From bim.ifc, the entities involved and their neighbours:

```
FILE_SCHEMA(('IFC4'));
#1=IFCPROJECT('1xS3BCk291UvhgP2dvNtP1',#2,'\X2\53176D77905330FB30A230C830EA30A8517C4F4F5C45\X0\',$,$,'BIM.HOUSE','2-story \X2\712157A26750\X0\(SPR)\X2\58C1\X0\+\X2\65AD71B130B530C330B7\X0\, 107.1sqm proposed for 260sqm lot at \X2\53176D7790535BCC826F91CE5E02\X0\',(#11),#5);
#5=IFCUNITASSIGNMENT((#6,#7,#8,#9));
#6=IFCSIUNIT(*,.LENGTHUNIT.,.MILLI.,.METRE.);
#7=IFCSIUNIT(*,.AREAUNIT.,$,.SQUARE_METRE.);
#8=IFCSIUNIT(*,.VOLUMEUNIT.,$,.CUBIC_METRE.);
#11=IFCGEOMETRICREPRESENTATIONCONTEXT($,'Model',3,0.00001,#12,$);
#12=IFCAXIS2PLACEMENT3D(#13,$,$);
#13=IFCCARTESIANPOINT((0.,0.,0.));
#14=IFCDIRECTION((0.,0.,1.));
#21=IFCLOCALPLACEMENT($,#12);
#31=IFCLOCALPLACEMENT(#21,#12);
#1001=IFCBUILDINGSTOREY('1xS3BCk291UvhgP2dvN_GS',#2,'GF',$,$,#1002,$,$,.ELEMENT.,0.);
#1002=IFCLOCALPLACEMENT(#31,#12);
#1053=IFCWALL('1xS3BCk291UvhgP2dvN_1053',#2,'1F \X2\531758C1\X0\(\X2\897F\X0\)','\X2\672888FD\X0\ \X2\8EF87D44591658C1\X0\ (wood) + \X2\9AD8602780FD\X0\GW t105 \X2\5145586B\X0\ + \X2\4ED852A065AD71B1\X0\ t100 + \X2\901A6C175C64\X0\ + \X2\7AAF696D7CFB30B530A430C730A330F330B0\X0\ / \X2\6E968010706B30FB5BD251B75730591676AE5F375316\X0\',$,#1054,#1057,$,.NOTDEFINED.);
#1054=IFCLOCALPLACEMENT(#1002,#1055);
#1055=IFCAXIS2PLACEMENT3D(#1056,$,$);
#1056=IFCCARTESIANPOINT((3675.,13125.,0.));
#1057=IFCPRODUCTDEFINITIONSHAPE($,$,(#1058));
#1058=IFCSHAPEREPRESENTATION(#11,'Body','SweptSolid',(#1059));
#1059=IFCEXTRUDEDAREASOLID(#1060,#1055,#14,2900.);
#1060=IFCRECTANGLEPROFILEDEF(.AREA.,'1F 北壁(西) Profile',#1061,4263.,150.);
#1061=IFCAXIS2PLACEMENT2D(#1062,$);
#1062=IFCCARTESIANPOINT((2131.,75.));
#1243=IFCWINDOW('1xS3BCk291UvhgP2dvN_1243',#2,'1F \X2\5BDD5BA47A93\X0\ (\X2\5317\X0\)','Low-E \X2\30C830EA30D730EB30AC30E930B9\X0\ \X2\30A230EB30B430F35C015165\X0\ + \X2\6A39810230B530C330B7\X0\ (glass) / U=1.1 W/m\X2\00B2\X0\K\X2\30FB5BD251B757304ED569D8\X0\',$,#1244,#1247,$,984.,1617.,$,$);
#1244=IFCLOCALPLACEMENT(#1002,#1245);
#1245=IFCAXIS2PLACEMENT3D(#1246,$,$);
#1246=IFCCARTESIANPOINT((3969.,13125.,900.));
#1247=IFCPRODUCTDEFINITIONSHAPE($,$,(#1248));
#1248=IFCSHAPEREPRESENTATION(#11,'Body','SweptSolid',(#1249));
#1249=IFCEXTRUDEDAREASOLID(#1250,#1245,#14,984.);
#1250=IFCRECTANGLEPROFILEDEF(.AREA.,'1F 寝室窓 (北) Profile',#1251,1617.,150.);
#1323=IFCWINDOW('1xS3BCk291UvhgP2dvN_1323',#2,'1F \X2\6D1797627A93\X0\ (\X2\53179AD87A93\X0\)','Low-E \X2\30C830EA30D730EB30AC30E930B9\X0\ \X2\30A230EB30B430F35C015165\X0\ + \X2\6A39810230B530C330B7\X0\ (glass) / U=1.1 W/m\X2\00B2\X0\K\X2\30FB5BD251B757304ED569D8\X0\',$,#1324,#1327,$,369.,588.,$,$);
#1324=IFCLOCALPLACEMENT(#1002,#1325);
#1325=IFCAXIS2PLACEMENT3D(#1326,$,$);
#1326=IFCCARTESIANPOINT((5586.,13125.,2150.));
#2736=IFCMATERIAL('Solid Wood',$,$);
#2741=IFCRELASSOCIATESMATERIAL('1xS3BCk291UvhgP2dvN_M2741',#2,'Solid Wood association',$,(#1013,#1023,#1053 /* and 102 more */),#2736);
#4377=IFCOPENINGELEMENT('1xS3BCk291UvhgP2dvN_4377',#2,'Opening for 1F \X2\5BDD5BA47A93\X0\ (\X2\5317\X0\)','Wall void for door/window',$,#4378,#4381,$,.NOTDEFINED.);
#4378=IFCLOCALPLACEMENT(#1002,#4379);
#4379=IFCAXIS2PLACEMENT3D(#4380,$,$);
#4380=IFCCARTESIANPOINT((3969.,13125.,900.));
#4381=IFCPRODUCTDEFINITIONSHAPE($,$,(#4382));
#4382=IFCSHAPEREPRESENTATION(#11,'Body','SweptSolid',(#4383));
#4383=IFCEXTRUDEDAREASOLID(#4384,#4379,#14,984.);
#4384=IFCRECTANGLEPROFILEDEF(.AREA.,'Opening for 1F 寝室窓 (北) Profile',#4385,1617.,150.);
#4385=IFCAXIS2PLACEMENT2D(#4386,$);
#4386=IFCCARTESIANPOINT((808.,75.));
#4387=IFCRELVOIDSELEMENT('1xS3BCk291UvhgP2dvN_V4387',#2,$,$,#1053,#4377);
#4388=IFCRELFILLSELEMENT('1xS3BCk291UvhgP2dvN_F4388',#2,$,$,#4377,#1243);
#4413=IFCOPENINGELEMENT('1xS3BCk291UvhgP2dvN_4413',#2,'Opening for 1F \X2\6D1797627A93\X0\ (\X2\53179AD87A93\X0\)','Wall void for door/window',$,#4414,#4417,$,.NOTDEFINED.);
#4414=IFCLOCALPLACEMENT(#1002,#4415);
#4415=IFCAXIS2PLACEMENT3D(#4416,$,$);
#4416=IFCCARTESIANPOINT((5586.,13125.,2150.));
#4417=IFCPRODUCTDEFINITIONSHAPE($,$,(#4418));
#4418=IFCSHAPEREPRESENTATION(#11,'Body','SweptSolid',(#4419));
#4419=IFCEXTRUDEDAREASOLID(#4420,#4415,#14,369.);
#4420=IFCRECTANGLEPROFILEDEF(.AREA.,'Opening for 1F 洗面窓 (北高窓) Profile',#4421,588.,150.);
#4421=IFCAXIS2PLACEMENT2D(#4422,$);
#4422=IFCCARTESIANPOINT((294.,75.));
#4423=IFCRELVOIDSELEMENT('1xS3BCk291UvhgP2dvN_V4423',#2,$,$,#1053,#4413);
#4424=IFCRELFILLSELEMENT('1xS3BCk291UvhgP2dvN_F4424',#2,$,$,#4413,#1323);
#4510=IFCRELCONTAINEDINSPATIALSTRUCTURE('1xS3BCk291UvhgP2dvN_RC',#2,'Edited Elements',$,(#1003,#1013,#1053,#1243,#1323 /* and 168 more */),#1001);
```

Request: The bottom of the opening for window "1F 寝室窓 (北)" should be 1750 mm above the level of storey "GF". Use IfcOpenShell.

```python
import numpy as np
import ifcopenshell
import ifcopenshell.api.geometry
import ifcopenshell.geom
import ifcopenshell.util.element
import ifcopenshell.util.placement
import ifcopenshell.util.shape
import ifcopenshell.util.unit

model = ifcopenshell.open("bim.ifc")
unit_scale = ifcopenshell.util.unit.calculate_unit_scale(model)

window = model.by_guid("1xS3BCk291UvhgP2dvN_1243")
opening = window.FillsVoids[0].RelatingOpeningElement
storey = ifcopenshell.util.element.get_container(window, ifc_class="IfcBuildingStorey")
level = ifcopenshell.util.placement.get_local_placement(storey.ObjectPlacement)[2, 3]

# The opening's origin need not be at the sill, so measure its lowest point.
shape = ifcopenshell.geom.create_shape(ifcopenshell.geom.settings(), opening)
bottom = ifcopenshell.util.shape.get_shape_bottom_elevation(shape, shape.geometry) / unit_scale
dz = level + 1750.0 - bottom

shift = np.array([0.0, 0.0, dz])
# The window is not placed relative to its opening, so move both.
for product in (opening, window):
    matrix = ifcopenshell.util.placement.get_local_placement(product.ObjectPlacement)
    matrix[:3, 3] += shift
    ifcopenshell.api.geometry.edit_object_placement(model, product=product, matrix=matrix, is_si=False)

print(f"moved by {dz * unit_scale:+.3f} m")

model.write("bim_rev.ifc")
```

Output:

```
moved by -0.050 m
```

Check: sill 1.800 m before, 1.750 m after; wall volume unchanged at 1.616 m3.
